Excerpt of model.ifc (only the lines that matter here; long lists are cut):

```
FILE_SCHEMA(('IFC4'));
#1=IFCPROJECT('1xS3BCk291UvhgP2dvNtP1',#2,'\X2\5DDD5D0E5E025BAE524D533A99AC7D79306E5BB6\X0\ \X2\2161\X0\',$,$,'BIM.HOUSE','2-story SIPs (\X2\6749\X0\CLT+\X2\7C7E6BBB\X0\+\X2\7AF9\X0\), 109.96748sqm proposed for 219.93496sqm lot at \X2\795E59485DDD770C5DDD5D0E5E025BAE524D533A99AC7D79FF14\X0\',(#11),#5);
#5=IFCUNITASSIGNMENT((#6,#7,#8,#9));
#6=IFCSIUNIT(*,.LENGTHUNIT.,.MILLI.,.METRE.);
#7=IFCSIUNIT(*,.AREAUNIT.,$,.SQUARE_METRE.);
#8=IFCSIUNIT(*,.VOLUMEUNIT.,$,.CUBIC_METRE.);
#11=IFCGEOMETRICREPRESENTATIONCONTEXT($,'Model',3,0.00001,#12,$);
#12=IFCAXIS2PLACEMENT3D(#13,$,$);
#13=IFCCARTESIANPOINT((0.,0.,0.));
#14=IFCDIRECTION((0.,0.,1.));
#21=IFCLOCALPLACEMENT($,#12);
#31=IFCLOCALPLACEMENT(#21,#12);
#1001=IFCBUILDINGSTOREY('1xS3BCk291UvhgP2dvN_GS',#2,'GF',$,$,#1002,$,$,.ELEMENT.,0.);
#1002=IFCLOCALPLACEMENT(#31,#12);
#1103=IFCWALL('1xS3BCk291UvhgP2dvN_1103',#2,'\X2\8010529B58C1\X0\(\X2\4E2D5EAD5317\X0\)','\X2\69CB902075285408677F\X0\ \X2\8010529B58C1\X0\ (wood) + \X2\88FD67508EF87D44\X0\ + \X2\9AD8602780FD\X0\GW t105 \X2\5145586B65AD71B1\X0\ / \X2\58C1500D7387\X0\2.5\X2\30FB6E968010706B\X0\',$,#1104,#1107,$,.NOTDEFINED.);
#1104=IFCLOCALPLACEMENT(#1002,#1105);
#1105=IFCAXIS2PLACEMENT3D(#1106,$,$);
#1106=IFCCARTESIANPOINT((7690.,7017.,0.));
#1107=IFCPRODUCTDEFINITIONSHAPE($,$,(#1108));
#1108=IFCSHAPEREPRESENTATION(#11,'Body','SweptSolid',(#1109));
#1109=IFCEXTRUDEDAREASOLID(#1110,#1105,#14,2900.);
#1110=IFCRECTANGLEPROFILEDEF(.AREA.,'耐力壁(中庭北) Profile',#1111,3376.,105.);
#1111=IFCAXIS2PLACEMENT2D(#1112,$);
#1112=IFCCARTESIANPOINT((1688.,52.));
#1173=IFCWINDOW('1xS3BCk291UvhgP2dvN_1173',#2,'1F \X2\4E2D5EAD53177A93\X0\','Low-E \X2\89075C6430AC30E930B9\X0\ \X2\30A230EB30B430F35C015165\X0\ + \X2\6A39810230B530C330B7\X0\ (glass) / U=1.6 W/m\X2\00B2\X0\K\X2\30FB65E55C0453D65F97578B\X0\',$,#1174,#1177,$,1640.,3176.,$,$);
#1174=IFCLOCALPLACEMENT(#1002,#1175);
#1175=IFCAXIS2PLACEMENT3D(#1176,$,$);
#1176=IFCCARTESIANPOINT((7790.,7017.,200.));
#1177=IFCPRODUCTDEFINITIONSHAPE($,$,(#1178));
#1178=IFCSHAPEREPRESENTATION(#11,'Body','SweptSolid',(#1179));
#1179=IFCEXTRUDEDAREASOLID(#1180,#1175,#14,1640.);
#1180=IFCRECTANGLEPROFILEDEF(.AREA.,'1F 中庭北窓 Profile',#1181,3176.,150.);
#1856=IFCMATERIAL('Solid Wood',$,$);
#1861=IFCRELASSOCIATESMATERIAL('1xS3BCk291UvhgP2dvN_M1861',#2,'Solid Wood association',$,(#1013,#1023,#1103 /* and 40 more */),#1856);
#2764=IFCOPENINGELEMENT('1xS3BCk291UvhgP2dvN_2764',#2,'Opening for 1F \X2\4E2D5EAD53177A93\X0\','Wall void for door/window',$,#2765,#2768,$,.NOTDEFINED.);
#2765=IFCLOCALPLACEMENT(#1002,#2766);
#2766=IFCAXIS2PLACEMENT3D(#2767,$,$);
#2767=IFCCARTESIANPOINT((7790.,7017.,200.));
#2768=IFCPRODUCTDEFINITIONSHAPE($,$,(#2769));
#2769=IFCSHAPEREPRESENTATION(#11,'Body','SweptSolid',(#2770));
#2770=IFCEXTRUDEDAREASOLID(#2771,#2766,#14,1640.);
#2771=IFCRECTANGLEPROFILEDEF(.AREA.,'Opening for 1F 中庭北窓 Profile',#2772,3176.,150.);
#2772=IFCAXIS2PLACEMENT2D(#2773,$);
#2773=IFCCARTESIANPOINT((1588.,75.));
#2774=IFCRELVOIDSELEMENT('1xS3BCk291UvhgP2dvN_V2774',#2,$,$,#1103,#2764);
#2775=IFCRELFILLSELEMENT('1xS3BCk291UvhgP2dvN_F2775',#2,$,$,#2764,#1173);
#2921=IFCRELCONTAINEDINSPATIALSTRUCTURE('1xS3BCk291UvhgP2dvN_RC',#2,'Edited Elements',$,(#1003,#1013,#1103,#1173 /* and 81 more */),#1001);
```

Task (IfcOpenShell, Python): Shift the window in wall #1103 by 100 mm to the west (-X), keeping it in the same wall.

```python
import ifcopenshell
import ifcopenshell.api.geometry
import ifcopenshell.util.placement
import ifcopenshell.util.unit

model = ifcopenshell.open("model.ifc")
unit_scale = ifcopenshell.util.unit.calculate_unit_scale(model)

window = model.by_guid("1xS3BCk291UvhgP2dvN_1173")
opening = window.FillsVoids[0].RelatingOpeningElement
wall = opening.VoidsElements[0].RelatingBuildingElement

wall_matrix = ifcopenshell.util.placement.get_local_placement(wall.ObjectPlacement)
shift = wall_matrix[:3, 0] * -0.1 / unit_scale
before = ifcopenshell.util.placement.get_local_placement(window.ObjectPlacement)[:3, 3].copy()

# The window is not placed relative to its opening, so move both.
for product in (opening, window):
    matrix = ifcopenshell.util.placement.get_local_placement(product.ObjectPlacement)
    matrix[:3, 3] += shift
    ifcopenshell.api.geometry.edit_object_placement(model, product=product, matrix=matrix, is_si=False)

after = ifcopenshell.util.placement.get_local_placement(window.ObjectPlacement)[:3, 3]
print("window moved by", (after - before).round(3) + 0.0)

model.write("model-out.ifc")
```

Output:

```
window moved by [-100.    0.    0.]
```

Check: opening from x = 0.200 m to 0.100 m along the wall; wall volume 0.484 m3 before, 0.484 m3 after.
